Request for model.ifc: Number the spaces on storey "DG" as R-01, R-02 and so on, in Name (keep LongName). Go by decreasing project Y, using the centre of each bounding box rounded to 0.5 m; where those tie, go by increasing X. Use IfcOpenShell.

First a look at what the model holds.

```python
import ifcopenshell
import ifcopenshell.util.element
import ifcopenshell.util.placement

model = ifcopenshell.open("model.ifc")
print(model.schema)
storey = next(s for s in model.by_type("IfcBuildingStorey") if s.Name == "DG")
spaces = [e for e in ifcopenshell.util.element.get_decomposition(storey) if e.is_a("IfcSpace")]
for e in sorted(spaces, key=lambda e: e.id()):
    origin = ifcopenshell.util.placement.get_local_placement(e.ObjectPlacement)[:3, 3]
    print(e.id(), e.Name, e.LongName, origin.round(2) + 0.0, sep=" | ")
```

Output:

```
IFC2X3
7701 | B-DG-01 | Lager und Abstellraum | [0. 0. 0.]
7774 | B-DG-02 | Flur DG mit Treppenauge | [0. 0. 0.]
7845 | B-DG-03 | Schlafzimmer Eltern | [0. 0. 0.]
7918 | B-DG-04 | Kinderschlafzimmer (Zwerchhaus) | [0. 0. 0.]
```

```python
import ifcopenshell
import ifcopenshell.geom
import ifcopenshell.util.element
import ifcopenshell.util.shape

model = ifcopenshell.open("model.ifc")
settings = ifcopenshell.geom.settings()
settings.set("use-world-coords", True)


def centre(element):
    shape = ifcopenshell.geom.create_shape(settings, element)
    return ifcopenshell.util.shape.get_bbox_centroid(shape.geometry)


storey = next(s for s in model.by_type("IfcBuildingStorey") if s.Name == "DG")
spaces = [e for e in ifcopenshell.util.element.get_decomposition(storey) if e.is_a("IfcSpace")]

# Insertion points can sit at a corner or the storey origin, so sort by the geometry (in metres).
centres = {e: centre(e) for e in spaces}
spaces.sort(key=lambda e: (-round(centres[e][1] / 0.5), centres[e][0]))

for i, e in enumerate(spaces, start=1):
    number = f"R-{i:02d}"
    e.Name = number
    print(e.id(), number)

model.write("model_updated.ifc")
```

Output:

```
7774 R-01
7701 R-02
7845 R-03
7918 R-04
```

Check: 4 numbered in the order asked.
